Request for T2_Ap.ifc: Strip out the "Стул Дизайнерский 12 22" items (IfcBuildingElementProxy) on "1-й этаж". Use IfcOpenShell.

First a look at what the model holds.

```python
import ifcopenshell
import ifcopenshell.util.element

model = ifcopenshell.open("T2_Ap.ifc")
print(model.schema)
storey = next(s for s in model.by_type("IfcBuildingStorey") if s.Name == "1-й этаж")
proxies = [e for e in ifcopenshell.util.element.get_decomposition(storey) if e.is_a("IfcBuildingElementProxy")]
seen = {}
for e in proxies:
    element_type = ifcopenshell.util.element.get_type(e)
    name = element_type.Name if element_type not in (None, e) else None
    seen[name] = seen.get(name, 0) + 1
for name, count in sorted(seen.items(), key=str):
    print(count, "x", name)
```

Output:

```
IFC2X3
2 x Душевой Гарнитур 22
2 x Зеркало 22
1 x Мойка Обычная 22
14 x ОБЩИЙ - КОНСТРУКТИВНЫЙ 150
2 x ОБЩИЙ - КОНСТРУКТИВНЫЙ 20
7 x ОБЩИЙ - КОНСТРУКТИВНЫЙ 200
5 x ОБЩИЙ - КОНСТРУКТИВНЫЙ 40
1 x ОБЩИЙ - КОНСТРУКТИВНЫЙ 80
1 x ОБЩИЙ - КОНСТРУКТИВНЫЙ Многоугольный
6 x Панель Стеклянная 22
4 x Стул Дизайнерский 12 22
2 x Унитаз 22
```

```python
import ifcopenshell
import ifcopenshell.api.root
import ifcopenshell.util.element

model = ifcopenshell.open("T2_Ap.ifc")

storey = next(s for s in model.by_type("IfcBuildingStorey") if s.Name == "1-й этаж")
proxies = [e for e in ifcopenshell.util.element.get_decomposition(storey) if e.is_a("IfcBuildingElementProxy")]
targets = [e for e in proxies if (t := ifcopenshell.util.element.get_type(e)) not in (None, e) and t.Name == "Стул Дизайнерский 12 22"]

for e in targets:
    ifcopenshell.api.root.remove_product(model, product=e)
print(len(targets), "removed")

model.write("T2_Ap_updated.ifc")
```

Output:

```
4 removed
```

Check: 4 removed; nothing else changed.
